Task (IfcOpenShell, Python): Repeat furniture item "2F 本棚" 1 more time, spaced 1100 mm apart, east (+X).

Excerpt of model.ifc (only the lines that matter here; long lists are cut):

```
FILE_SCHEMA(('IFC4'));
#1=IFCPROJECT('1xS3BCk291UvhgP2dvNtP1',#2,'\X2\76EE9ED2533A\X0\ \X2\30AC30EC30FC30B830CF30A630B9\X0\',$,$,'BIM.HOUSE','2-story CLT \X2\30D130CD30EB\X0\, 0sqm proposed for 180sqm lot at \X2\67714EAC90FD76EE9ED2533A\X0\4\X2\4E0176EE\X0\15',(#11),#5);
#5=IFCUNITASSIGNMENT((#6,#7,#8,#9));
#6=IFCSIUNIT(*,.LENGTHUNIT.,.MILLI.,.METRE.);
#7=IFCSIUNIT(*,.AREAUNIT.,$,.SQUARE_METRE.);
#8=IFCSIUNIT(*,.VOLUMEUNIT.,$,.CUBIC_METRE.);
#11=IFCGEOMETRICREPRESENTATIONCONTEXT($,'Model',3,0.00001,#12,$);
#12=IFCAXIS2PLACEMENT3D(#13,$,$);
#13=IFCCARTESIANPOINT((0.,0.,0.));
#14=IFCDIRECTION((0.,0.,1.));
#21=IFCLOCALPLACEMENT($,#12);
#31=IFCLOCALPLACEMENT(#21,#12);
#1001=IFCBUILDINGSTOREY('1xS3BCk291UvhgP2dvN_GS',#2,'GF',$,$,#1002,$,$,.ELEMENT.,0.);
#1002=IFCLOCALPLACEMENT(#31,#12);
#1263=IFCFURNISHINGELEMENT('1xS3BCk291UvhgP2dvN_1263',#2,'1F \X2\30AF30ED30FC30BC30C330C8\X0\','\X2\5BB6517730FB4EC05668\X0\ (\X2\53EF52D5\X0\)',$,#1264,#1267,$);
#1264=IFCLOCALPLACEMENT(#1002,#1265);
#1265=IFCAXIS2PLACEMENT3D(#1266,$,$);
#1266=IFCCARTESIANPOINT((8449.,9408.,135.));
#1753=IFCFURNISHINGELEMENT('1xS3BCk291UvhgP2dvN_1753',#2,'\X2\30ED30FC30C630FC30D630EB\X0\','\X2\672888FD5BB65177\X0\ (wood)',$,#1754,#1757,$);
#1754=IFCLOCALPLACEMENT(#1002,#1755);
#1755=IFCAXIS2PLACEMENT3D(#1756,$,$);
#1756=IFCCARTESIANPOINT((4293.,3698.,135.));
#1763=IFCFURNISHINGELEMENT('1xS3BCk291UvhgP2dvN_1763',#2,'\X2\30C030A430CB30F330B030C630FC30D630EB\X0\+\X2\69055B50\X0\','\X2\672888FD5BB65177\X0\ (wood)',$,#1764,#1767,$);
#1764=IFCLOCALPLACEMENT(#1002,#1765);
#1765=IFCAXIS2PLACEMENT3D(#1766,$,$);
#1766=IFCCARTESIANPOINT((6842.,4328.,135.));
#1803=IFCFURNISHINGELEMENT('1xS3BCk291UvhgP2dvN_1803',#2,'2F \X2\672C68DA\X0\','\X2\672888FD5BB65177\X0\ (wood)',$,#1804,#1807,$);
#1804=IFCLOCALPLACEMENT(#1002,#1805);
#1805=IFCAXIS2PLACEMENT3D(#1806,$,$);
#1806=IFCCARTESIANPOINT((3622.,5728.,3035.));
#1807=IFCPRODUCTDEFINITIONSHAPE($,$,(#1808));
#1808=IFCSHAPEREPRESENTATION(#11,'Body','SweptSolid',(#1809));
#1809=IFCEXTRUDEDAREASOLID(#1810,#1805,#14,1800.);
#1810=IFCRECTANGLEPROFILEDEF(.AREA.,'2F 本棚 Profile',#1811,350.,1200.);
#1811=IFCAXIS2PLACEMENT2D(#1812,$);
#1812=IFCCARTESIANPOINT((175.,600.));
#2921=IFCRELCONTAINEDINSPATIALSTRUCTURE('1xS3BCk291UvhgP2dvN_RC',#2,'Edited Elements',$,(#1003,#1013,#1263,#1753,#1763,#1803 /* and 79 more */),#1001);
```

```python
import numpy as np
import ifcopenshell
import ifcopenshell.api.geometry
import ifcopenshell.api.root
import ifcopenshell.util.element
import ifcopenshell.util.placement
import ifcopenshell.util.unit

model = ifcopenshell.open("model.ifc")
unit_scale = ifcopenshell.util.unit.calculate_unit_scale(model)


def reuse_history(source, copy):
    """copy_class also copies each property set's owner history, people and application; keep the originals."""
    for rel in copy.IsDefinedBy:
        if rel.is_a("IfcRelDefinesByProperties") and (history := rel.RelatingPropertyDefinition.OwnerHistory):
            rel.RelatingPropertyDefinition.OwnerHistory = source.OwnerHistory
            ifcopenshell.util.element.remove_deep2(model, history)


source = model.by_id(1803)
base = ifcopenshell.util.placement.get_local_placement(source.ObjectPlacement)
step = np.array([1.0, 0.0, 0.0]) * 1.1 / unit_scale

for i in range(1, 2):
    copy = ifcopenshell.api.root.copy_class(model, product=source)
    copy.Representation = ifcopenshell.util.element.copy_deep(
        model, source.Representation, exclude=["IfcGeometricRepresentationContext", "IfcRepresentationMap"]
    )
    reuse_history(source, copy)
    matrix = base.copy()
    matrix[:3, 3] += i * step
    print("added at", matrix[:3, 3].round(3) + 0.0)
    ifcopenshell.api.geometry.edit_object_placement(model, product=copy, matrix=matrix, is_si=False)

model.write("model-out.ifc")
```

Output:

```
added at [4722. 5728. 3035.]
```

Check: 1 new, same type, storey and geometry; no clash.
